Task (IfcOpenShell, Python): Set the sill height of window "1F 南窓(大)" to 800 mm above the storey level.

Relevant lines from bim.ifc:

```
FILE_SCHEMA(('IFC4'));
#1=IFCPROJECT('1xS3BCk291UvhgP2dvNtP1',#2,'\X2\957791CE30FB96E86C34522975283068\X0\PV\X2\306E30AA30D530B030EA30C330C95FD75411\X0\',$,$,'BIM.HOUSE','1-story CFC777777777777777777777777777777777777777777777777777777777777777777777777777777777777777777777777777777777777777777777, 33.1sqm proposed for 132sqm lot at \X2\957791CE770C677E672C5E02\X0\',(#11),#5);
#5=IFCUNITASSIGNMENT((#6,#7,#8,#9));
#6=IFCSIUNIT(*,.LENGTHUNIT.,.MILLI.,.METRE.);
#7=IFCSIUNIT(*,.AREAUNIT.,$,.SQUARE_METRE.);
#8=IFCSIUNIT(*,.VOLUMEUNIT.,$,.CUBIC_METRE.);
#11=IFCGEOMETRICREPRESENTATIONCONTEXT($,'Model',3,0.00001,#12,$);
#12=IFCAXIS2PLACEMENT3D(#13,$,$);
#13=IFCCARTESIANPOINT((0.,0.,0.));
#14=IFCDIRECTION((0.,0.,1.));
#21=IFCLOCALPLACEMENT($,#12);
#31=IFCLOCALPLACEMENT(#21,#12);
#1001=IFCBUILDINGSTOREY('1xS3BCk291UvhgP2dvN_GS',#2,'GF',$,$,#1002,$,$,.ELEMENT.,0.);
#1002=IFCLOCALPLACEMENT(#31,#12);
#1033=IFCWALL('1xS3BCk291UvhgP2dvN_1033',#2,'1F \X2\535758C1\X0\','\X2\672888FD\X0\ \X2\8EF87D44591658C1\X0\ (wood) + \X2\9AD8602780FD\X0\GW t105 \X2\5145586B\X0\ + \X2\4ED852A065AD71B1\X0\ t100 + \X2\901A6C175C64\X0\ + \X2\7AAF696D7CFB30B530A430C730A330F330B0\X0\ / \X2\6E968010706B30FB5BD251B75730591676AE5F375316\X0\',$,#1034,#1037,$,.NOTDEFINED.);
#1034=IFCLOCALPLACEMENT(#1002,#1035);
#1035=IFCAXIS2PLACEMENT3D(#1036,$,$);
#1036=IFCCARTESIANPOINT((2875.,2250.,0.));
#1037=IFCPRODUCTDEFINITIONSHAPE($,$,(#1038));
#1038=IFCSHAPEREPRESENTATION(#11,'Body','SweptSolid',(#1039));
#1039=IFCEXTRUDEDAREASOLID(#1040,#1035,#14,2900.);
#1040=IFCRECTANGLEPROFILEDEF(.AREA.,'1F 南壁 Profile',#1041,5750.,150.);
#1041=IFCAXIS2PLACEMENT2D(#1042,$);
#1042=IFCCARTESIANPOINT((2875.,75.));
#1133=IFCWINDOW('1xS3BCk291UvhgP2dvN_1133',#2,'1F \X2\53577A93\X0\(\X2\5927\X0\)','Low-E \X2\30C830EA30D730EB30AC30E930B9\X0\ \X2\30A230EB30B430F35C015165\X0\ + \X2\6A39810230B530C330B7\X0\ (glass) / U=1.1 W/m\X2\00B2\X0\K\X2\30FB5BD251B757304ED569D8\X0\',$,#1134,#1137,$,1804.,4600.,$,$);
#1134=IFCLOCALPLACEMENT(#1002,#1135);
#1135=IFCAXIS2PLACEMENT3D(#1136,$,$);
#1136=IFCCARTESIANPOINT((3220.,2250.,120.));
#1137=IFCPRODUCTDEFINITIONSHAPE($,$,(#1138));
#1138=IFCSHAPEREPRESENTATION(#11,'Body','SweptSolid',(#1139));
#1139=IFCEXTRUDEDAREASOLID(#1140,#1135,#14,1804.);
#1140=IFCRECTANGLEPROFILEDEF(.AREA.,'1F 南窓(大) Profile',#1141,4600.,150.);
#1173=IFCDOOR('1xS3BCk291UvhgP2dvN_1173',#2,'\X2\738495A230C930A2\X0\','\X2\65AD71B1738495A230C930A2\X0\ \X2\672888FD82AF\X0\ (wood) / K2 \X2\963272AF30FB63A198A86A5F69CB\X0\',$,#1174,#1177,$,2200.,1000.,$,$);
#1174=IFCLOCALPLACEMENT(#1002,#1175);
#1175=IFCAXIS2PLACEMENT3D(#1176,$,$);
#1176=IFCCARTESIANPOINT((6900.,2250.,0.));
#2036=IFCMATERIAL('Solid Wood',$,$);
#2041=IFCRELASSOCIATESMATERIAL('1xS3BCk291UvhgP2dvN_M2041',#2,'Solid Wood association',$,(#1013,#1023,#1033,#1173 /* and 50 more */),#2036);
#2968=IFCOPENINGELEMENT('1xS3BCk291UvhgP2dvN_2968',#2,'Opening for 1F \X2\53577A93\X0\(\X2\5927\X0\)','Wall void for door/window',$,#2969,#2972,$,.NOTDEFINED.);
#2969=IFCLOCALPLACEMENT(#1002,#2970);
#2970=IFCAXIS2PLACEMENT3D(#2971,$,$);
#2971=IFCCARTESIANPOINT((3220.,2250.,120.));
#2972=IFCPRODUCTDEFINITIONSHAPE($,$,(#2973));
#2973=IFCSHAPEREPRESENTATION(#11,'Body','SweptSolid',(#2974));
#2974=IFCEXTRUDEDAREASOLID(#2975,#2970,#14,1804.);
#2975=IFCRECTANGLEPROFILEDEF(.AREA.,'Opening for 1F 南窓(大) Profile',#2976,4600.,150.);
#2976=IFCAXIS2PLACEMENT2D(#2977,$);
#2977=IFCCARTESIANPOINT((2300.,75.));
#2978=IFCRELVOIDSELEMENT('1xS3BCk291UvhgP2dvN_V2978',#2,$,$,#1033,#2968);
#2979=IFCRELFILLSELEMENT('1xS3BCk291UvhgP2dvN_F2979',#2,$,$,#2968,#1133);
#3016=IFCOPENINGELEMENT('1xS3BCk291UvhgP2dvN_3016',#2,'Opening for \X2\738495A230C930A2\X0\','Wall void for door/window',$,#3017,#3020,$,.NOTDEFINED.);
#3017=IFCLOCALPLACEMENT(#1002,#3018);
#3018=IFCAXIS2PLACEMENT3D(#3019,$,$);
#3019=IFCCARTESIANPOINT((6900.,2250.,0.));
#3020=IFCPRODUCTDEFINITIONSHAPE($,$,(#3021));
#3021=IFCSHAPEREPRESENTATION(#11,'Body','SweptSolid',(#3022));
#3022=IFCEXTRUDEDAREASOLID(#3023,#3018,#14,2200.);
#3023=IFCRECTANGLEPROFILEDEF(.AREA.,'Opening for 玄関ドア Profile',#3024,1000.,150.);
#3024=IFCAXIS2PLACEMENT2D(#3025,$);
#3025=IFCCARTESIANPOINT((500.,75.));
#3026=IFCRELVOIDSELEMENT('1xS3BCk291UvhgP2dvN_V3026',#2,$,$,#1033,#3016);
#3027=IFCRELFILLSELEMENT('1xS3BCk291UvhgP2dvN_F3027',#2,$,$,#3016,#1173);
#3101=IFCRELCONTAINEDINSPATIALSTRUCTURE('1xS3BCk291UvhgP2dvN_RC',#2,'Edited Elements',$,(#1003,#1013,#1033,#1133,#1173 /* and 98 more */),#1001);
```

```python
import numpy as np
import ifcopenshell
import ifcopenshell.api.geometry
import ifcopenshell.geom
import ifcopenshell.util.element
import ifcopenshell.util.placement
import ifcopenshell.util.shape
import ifcopenshell.util.unit

model = ifcopenshell.open("bim.ifc")
unit_scale = ifcopenshell.util.unit.calculate_unit_scale(model)

window = model.by_id(1133)
opening = window.FillsVoids[0].RelatingOpeningElement
storey = ifcopenshell.util.element.get_container(window, ifc_class="IfcBuildingStorey")
level = ifcopenshell.util.placement.get_local_placement(storey.ObjectPlacement)[2, 3]

# The opening's origin need not be at the sill, so measure its lowest point.
shape = ifcopenshell.geom.create_shape(ifcopenshell.geom.settings(), opening)
bottom = ifcopenshell.util.shape.get_shape_bottom_elevation(shape, shape.geometry) / unit_scale
dz = level + 0.8 / unit_scale - bottom

shift = np.array([0.0, 0.0, dz])
# The window is not placed relative to its opening, so move both.
for product in (opening, window):
    matrix = ifcopenshell.util.placement.get_local_placement(product.ObjectPlacement)
    matrix[:3, 3] += shift
    ifcopenshell.api.geometry.edit_object_placement(model, product=product, matrix=matrix, is_si=False)

print(f"moved by {dz * unit_scale:+.3f} m")

model.write("bim_rev.ifc")
```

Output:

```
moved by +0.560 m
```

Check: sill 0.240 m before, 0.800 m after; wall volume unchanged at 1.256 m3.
